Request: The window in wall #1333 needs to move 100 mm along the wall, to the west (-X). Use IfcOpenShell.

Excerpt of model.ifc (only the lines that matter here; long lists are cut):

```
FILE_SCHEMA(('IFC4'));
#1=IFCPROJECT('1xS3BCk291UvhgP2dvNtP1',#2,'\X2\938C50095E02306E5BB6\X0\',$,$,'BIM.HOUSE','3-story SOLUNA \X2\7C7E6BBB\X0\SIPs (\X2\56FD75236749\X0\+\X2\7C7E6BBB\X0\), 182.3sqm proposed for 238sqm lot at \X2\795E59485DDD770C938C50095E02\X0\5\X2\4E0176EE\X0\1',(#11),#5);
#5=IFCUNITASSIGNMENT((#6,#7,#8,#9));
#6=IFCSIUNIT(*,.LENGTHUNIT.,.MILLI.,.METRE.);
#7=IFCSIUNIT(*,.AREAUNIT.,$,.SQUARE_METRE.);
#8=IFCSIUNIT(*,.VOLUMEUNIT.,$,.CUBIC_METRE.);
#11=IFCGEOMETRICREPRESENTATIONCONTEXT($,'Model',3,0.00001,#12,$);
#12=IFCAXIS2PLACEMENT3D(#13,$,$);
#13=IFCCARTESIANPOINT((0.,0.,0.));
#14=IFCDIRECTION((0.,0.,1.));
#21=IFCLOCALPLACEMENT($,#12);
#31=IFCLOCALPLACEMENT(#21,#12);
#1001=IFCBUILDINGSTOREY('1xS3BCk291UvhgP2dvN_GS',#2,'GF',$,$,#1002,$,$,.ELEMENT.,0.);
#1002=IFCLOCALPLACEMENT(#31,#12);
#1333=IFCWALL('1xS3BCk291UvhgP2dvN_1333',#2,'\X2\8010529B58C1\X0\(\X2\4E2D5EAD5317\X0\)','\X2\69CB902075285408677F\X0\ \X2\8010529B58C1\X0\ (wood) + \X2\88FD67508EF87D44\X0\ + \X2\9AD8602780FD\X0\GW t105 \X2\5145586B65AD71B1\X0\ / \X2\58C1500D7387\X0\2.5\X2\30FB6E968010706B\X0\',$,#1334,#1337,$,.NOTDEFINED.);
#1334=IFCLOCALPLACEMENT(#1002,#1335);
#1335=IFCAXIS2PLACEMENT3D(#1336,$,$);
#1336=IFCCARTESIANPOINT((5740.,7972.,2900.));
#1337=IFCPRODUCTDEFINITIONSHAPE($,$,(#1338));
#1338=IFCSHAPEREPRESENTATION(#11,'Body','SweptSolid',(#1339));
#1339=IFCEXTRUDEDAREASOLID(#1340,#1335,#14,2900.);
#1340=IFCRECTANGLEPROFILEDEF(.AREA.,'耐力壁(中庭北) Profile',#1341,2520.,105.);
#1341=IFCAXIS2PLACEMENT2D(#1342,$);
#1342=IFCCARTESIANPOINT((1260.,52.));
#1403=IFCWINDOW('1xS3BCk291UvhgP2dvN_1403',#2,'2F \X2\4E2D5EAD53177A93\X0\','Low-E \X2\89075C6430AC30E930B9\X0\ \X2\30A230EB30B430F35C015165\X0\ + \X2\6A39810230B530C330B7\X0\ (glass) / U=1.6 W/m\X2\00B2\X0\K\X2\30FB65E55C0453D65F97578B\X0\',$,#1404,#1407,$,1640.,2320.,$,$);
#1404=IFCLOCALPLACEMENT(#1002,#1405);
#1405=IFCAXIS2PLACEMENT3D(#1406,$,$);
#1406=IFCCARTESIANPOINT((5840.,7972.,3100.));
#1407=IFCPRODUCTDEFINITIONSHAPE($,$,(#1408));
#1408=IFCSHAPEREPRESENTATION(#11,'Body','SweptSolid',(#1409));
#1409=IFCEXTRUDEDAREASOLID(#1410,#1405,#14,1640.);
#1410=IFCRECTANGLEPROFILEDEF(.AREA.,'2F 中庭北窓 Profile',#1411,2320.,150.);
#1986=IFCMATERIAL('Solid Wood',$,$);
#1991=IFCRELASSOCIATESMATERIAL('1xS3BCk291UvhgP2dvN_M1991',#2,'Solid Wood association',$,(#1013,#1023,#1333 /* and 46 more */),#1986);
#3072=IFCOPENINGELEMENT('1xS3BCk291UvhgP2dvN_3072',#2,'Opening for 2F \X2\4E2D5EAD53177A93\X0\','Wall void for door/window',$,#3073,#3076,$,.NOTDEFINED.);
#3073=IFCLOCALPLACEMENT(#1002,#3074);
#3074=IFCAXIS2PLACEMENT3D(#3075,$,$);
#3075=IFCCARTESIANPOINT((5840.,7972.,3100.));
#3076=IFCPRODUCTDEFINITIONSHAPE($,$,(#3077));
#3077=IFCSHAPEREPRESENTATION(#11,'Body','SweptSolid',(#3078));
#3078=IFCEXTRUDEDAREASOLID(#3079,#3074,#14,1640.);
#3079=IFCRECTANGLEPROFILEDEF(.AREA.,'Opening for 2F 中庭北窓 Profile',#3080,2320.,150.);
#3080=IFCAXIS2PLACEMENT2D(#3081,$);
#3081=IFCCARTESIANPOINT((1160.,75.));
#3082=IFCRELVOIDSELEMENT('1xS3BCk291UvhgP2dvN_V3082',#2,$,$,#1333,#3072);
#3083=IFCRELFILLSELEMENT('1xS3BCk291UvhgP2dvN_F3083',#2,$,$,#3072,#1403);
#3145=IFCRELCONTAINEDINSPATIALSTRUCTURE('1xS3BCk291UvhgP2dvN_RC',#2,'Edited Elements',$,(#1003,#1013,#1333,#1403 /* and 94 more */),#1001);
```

```python
import ifcopenshell
import ifcopenshell.api.geometry
import ifcopenshell.util.placement

model = ifcopenshell.open("model.ifc")

window = model.by_guid("1xS3BCk291UvhgP2dvN_1403")
opening = window.FillsVoids[0].RelatingOpeningElement
wall = opening.VoidsElements[0].RelatingBuildingElement

wall_matrix = ifcopenshell.util.placement.get_local_placement(wall.ObjectPlacement)
shift = wall_matrix[:3, 0] * -100.0
before = ifcopenshell.util.placement.get_local_placement(window.ObjectPlacement)[:3, 3].copy()

# The window is not placed relative to its opening, so move both.
for product in (opening, window):
    matrix = ifcopenshell.util.placement.get_local_placement(product.ObjectPlacement)
    matrix[:3, 3] += shift
    ifcopenshell.api.geometry.edit_object_placement(model, product=product, matrix=matrix, is_si=False)

after = ifcopenshell.util.placement.get_local_placement(window.ObjectPlacement)[:3, 3]
print("window moved by", (after - before).round(3) + 0.0)

model.write("model_updated.ifc")
```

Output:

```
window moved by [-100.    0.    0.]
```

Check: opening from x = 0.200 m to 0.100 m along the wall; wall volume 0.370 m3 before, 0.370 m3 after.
